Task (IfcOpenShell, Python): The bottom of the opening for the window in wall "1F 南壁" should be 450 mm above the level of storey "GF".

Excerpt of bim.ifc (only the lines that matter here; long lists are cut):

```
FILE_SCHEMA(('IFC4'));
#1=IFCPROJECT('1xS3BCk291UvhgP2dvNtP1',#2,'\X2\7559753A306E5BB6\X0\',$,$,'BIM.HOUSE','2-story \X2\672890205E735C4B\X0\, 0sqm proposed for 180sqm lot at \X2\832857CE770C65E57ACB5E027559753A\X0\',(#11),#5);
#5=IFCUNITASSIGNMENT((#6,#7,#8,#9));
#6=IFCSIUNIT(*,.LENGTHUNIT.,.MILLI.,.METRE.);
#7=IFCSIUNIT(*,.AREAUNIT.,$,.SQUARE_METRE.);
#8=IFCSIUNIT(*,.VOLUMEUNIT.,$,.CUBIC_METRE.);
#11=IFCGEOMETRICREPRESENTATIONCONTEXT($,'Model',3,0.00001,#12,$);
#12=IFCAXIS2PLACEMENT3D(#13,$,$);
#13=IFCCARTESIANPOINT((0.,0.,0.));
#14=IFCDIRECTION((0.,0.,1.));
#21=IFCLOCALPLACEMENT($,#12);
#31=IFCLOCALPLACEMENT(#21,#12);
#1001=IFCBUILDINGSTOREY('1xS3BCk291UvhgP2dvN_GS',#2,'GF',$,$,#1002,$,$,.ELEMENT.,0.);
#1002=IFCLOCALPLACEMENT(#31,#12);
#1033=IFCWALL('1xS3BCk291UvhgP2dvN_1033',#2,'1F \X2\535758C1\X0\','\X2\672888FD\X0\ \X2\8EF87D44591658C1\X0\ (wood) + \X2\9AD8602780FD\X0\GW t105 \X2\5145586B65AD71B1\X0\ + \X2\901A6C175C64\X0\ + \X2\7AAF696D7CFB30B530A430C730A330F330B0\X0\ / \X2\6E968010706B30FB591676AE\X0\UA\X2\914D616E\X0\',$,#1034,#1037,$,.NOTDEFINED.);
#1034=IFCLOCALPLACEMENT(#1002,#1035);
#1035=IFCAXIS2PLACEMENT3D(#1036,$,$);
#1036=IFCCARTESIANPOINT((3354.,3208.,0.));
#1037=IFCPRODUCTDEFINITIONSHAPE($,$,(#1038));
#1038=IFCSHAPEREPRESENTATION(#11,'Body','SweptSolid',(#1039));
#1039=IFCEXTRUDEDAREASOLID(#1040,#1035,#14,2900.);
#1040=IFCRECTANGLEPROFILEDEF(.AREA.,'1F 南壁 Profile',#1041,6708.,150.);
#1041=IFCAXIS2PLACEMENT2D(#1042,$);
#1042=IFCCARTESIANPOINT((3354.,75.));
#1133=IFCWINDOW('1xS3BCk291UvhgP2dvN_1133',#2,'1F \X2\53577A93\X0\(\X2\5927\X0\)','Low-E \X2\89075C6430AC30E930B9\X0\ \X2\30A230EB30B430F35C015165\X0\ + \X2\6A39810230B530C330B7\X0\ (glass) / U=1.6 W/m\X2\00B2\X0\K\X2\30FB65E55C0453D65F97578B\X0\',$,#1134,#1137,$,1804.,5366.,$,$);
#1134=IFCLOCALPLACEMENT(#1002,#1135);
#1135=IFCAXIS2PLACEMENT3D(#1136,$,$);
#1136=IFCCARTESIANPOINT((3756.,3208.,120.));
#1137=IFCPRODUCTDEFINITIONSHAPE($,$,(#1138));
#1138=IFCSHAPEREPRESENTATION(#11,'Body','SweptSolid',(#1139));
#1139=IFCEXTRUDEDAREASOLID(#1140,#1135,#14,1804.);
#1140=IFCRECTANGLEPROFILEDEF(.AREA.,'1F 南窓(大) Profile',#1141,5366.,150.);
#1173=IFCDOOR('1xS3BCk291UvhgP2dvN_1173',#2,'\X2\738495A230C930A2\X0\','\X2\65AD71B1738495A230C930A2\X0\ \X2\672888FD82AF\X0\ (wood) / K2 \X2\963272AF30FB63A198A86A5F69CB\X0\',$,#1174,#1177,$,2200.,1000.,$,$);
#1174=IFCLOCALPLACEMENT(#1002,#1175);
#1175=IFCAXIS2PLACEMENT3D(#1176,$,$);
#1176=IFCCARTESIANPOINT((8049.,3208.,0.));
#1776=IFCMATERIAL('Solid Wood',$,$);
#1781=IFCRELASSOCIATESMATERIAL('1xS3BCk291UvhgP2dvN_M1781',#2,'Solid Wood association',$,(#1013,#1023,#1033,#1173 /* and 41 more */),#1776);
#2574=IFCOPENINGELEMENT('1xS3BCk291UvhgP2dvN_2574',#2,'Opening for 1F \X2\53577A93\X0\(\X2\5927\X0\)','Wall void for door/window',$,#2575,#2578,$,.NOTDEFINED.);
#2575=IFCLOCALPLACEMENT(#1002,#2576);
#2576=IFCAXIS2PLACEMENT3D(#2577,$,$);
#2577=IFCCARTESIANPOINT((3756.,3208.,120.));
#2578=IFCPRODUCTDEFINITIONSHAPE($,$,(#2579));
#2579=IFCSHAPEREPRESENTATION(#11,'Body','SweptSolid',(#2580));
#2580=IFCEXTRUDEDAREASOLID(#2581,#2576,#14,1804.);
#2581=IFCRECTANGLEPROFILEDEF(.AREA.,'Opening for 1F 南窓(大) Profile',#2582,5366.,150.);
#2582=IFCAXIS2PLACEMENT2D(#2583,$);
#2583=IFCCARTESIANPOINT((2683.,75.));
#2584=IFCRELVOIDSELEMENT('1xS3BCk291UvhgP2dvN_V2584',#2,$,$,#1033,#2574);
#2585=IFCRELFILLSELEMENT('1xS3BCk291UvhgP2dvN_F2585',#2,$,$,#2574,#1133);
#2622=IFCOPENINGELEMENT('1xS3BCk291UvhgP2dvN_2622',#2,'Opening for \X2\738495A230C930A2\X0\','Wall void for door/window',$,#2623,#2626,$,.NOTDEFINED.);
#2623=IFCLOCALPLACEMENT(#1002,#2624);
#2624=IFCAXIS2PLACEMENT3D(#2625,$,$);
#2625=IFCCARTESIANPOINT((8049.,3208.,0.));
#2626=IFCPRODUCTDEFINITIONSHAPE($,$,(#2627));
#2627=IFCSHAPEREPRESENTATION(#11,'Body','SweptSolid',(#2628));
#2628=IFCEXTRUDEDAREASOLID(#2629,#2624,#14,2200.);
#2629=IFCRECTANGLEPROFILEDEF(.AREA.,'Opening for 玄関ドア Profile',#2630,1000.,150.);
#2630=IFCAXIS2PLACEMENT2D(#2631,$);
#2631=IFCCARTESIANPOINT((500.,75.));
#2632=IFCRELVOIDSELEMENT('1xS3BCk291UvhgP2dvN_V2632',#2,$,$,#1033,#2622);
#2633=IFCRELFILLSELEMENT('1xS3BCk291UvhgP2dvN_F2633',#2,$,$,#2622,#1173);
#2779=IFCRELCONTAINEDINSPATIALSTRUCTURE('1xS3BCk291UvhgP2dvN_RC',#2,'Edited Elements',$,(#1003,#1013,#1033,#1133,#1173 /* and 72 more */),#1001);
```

```python
import numpy as np
import ifcopenshell
import ifcopenshell.api.geometry
import ifcopenshell.geom
import ifcopenshell.util.element
import ifcopenshell.util.placement
import ifcopenshell.util.shape
import ifcopenshell.util.unit

model = ifcopenshell.open("bim.ifc")
unit_scale = ifcopenshell.util.unit.calculate_unit_scale(model)

window = model.by_id(1133)
opening = window.FillsVoids[0].RelatingOpeningElement
storey = ifcopenshell.util.element.get_container(window, ifc_class="IfcBuildingStorey")
level = ifcopenshell.util.placement.get_local_placement(storey.ObjectPlacement)[2, 3]

# The opening's origin need not be at the sill, so measure its lowest point.
shape = ifcopenshell.geom.create_shape(ifcopenshell.geom.settings(), opening)
bottom = ifcopenshell.util.shape.get_shape_bottom_elevation(shape, shape.geometry) / unit_scale
dz = level + 0.45 / unit_scale - bottom

shift = np.array([0.0, 0.0, dz])
# The window is not placed relative to its opening, so move both.
for product in (opening, window):
    matrix = ifcopenshell.util.placement.get_local_placement(product.ObjectPlacement)
    matrix[:3, 3] += shift
    ifcopenshell.api.geometry.edit_object_placement(model, product=product, matrix=matrix, is_si=False)

print(f"moved by {dz * unit_scale:+.3f} m")

model.write("bim_v2.ifc")
```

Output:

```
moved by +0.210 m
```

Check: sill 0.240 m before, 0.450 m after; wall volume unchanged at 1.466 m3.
